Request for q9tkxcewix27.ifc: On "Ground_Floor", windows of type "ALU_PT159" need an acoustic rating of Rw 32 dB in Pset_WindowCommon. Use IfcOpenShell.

First a look at what the model holds.

```python
import ifcopenshell
import ifcopenshell.util.element

model = ifcopenshell.open("q9tkxcewix27.ifc")
print(model.schema)
storey = next(s for s in model.by_type("IfcBuildingStorey") if s.Name == "Ground_Floor")
windows = [e for e in ifcopenshell.util.element.get_decomposition(storey) if e.is_a("IfcWindow")]
seen = {}
for e in windows:
    element_type = ifcopenshell.util.element.get_type(e)
    key = (element_type.Name if element_type != e and element_type else None, ifcopenshell.util.element.get_pset(e, "Pset_WindowCommon", "AcousticRating"))
    seen[key] = seen.get(key, 0) + 1
for (name, value), count in sorted(seen.items(), key=str):
    print(count, "x", name, "|", value)
```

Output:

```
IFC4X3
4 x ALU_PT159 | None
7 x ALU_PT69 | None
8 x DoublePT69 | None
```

```python
import ifcopenshell
import ifcopenshell.api.pset
import ifcopenshell.util.element

model = ifcopenshell.open("q9tkxcewix27.ifc")

storey = next(s for s in model.by_type("IfcBuildingStorey") if s.Name == "Ground_Floor")
windows = [e for e in ifcopenshell.util.element.get_decomposition(storey) if e.is_a("IfcWindow")]

count = 0
for e in windows:
    element_type = ifcopenshell.util.element.get_type(e)
    if element_type in (None, e) or element_type.Name != "ALU_PT159":
        continue
    # add_pset returns the element's existing set when there is one.
    pset = ifcopenshell.api.pset.add_pset(model, product=e, name="Pset_WindowCommon")
    ifcopenshell.api.pset.edit_pset(model, pset=pset, properties={"AcousticRating": "Rw 32 dB"})
    count += 1

print(count, "windows updated")

model.write("q9tkxcewix27_edited.ifc")
```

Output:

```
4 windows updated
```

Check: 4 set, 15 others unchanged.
